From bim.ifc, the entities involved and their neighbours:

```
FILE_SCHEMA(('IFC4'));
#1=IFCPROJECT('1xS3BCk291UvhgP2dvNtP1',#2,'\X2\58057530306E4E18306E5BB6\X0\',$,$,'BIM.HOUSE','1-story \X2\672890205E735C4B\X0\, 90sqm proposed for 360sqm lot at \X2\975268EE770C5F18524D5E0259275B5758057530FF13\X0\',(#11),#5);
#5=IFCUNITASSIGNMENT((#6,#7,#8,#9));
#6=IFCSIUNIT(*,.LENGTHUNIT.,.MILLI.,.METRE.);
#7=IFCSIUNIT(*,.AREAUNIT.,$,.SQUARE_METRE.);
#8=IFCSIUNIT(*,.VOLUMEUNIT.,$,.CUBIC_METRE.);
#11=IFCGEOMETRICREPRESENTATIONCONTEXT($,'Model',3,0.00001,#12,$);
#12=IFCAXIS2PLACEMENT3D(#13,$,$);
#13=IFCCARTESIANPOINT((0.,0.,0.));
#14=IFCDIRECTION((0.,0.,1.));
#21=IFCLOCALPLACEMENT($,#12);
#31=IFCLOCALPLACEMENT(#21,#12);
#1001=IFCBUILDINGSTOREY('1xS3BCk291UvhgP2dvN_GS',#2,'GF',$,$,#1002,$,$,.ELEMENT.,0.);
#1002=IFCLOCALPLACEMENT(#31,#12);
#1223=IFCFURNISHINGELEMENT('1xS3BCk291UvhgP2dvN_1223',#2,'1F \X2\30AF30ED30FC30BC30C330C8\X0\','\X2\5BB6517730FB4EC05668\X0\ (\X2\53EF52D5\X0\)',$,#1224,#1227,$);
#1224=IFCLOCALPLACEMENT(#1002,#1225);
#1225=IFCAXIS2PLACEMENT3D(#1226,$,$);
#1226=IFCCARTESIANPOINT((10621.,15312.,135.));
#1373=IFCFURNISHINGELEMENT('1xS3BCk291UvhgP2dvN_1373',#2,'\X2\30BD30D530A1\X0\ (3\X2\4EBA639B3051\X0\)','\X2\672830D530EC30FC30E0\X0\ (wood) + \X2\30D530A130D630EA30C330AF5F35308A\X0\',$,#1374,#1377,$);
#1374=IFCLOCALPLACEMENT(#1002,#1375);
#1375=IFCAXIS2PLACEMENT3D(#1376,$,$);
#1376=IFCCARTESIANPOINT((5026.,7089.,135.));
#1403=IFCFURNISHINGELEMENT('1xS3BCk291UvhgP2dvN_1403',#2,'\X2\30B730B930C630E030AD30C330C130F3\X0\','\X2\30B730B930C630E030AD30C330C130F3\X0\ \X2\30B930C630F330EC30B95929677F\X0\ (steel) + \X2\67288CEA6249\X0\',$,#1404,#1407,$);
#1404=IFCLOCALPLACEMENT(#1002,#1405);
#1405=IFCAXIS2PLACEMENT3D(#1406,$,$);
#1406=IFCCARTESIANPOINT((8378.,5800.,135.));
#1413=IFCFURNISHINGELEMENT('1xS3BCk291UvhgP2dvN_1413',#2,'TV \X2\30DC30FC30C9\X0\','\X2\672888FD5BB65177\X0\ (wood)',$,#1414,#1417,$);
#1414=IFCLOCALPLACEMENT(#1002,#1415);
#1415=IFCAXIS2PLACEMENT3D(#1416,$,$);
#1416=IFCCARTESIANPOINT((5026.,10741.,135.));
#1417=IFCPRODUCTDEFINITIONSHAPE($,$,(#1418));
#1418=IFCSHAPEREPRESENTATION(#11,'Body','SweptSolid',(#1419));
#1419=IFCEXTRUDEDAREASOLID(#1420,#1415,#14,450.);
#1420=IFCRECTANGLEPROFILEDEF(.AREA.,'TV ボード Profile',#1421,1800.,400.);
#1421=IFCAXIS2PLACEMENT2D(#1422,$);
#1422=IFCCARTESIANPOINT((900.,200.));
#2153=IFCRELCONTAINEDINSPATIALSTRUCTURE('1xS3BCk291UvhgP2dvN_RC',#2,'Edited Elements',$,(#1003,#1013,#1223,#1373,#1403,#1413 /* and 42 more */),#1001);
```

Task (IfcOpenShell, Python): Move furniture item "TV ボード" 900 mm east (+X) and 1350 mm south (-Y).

```python
import ifcopenshell
import ifcopenshell.api.geometry
import ifcopenshell.util.placement

model = ifcopenshell.open("bim.ifc")

item = model.by_id(1413)
matrix = ifcopenshell.util.placement.get_local_placement(item.ObjectPlacement)
matrix[0, 3] += 900.0
matrix[1, 3] -= 1350.0
ifcopenshell.api.geometry.edit_object_placement(model, product=item, matrix=matrix, is_si=False)

print(ifcopenshell.util.placement.get_local_placement(item.ObjectPlacement).round(3) + 0.0)

model.write("bim_updated.ifc")
```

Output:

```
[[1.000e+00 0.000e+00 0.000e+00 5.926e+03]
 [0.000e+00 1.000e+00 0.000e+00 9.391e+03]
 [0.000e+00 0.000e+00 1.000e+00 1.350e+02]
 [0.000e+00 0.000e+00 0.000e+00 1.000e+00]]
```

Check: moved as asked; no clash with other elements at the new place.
